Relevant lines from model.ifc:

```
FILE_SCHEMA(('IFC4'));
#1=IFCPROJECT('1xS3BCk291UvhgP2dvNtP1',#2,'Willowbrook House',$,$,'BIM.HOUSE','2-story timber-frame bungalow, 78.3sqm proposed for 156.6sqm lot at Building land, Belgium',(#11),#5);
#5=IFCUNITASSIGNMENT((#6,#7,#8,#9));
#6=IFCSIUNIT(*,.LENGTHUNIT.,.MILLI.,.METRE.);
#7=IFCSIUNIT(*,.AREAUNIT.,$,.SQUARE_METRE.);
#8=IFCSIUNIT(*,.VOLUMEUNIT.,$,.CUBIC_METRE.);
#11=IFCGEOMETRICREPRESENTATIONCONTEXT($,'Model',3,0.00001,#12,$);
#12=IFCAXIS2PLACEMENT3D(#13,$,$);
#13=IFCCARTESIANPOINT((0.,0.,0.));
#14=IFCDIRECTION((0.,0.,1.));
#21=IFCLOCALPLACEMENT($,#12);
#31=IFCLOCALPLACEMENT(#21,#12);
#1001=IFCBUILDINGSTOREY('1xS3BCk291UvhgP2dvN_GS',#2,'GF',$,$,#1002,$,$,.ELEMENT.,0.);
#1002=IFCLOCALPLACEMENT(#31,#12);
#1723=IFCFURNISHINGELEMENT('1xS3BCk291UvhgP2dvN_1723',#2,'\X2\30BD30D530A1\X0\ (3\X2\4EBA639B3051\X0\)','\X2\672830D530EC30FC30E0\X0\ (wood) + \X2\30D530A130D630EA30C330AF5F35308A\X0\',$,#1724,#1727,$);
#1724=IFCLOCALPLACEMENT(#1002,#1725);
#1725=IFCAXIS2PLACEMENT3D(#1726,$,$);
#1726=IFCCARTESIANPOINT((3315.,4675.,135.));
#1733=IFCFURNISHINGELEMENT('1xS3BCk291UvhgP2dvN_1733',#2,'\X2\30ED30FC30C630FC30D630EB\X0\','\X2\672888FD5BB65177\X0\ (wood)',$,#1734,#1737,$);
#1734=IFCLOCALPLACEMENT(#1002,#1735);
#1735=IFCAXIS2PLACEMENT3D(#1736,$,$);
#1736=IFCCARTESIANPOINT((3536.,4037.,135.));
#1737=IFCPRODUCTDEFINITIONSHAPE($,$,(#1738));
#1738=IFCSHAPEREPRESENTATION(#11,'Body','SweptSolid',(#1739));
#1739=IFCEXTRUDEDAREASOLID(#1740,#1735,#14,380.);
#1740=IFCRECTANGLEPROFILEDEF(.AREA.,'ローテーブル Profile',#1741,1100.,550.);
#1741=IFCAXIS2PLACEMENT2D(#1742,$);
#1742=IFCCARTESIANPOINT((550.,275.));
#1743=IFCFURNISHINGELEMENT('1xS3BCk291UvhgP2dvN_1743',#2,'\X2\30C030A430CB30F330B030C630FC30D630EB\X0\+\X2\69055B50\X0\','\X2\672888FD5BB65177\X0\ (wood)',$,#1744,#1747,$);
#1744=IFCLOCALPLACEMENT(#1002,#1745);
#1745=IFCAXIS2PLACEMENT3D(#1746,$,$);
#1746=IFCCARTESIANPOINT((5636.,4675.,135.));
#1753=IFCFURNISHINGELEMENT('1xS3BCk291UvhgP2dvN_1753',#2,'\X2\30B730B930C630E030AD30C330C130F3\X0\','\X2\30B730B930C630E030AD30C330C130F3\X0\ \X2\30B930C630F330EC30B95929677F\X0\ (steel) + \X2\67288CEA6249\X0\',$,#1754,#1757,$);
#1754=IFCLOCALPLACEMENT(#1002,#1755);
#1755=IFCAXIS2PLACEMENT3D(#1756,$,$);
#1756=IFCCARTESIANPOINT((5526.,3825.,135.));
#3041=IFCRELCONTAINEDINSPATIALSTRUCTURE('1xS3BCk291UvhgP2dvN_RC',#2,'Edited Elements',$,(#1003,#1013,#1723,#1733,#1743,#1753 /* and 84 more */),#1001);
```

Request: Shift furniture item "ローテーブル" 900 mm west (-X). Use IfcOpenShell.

```python
import ifcopenshell
import ifcopenshell.api.geometry
import ifcopenshell.util.placement

model = ifcopenshell.open("model.ifc")

item = model.by_guid("1xS3BCk291UvhgP2dvN_1733")
matrix = ifcopenshell.util.placement.get_local_placement(item.ObjectPlacement)
matrix[0, 3] -= 900.0
ifcopenshell.api.geometry.edit_object_placement(model, product=item, matrix=matrix, is_si=False)

print(ifcopenshell.util.placement.get_local_placement(item.ObjectPlacement).round(3) + 0.0)

model.write("model_edited.ifc")
```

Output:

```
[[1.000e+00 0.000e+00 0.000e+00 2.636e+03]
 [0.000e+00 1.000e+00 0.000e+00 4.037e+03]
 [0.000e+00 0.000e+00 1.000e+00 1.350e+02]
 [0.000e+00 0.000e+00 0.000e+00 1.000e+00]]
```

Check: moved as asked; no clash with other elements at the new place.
